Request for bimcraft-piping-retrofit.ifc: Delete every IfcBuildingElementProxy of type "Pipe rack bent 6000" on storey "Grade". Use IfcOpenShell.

First a look at what the model holds.

```python
import ifcopenshell
import ifcopenshell.util.element

model = ifcopenshell.open("bimcraft-piping-retrofit.ifc")
print(model.schema)
storey = next(s for s in model.by_type("IfcBuildingStorey") if s.Name == "Grade")
proxies = [e for e in ifcopenshell.util.element.get_decomposition(storey) if e.is_a("IfcBuildingElementProxy")]
seen = {}
for e in proxies:
    element_type = ifcopenshell.util.element.get_type(e)
    name = element_type.Name if element_type not in (None, e) else None
    seen[name] = seen.get(name, 0) + 1
for name, count in sorted(seen.items(), key=str):
    print(count, "x", name)
```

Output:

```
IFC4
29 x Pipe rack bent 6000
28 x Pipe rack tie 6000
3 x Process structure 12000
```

```python
import ifcopenshell
import ifcopenshell.api.root
import ifcopenshell.util.element

model = ifcopenshell.open("bimcraft-piping-retrofit.ifc")

storey = next(s for s in model.by_type("IfcBuildingStorey") if s.Name == "Grade")
proxies = [e for e in ifcopenshell.util.element.get_decomposition(storey) if e.is_a("IfcBuildingElementProxy")]
targets = [e for e in proxies if (t := ifcopenshell.util.element.get_type(e)) not in (None, e) and t.Name == "Pipe rack bent 6000"]

for e in targets:
    ifcopenshell.api.root.remove_product(model, product=e)
print(len(targets), "removed")

model.write("bimcraft-piping-retrofit_edited.ifc")
```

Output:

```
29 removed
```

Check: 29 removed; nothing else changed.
